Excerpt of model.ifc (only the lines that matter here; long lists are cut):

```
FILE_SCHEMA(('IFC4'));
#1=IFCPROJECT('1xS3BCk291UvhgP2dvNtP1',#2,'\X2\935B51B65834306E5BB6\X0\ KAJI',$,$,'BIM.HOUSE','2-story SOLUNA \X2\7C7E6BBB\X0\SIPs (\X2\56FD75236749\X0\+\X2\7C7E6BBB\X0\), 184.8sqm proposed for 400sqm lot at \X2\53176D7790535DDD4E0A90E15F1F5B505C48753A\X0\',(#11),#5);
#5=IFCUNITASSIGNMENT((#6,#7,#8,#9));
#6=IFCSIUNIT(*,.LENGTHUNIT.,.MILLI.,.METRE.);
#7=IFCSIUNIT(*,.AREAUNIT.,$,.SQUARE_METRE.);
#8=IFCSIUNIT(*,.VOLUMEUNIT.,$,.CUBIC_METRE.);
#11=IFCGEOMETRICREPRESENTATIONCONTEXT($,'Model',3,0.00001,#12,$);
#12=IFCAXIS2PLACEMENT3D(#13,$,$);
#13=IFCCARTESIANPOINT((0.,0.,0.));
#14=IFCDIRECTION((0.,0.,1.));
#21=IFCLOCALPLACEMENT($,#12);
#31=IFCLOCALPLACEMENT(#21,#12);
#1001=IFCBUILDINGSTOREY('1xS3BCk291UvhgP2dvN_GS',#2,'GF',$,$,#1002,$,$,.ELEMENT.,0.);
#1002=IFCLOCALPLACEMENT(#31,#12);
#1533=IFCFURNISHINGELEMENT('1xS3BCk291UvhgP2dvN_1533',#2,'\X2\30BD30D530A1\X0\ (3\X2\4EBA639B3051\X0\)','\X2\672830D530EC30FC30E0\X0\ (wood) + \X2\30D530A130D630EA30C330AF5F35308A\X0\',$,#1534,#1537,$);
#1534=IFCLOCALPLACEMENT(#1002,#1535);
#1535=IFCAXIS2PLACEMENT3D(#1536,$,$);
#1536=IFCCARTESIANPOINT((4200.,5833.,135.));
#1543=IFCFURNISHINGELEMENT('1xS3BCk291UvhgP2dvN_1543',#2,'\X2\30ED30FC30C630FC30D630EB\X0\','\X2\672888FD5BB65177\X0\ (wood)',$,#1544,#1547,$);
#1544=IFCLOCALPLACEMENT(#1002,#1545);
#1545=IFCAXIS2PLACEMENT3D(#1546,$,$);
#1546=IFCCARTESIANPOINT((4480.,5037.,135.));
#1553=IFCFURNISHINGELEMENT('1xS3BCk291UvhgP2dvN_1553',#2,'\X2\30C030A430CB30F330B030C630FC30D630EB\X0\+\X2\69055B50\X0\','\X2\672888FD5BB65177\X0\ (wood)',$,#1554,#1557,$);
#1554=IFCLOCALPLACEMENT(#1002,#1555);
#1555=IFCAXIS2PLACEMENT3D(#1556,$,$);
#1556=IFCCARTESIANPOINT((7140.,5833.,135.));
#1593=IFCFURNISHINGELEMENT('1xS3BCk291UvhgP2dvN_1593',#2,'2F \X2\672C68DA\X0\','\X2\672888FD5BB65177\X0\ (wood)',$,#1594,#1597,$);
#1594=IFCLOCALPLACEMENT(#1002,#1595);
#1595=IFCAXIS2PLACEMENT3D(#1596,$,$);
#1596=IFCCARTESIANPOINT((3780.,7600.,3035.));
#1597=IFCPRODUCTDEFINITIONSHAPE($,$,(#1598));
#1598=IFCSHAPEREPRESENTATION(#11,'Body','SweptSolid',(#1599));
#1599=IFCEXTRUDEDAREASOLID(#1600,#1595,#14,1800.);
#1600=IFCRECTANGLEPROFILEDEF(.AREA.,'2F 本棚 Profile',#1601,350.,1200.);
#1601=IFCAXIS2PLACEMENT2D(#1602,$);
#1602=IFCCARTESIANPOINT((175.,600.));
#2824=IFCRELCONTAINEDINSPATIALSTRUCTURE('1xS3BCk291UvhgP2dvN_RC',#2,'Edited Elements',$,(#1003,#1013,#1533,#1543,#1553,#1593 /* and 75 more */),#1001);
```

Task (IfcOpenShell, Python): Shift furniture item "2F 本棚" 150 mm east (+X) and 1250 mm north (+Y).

```python
import ifcopenshell
import ifcopenshell.api.geometry
import ifcopenshell.util.placement

model = ifcopenshell.open("model.ifc")

item = model.by_guid("1xS3BCk291UvhgP2dvN_1593")
matrix = ifcopenshell.util.placement.get_local_placement(item.ObjectPlacement)
matrix[0, 3] += 150.0
matrix[1, 3] += 1250.0
ifcopenshell.api.geometry.edit_object_placement(model, product=item, matrix=matrix, is_si=False)

print(ifcopenshell.util.placement.get_local_placement(item.ObjectPlacement).round(3) + 0.0)

model.write("model-out.ifc")
```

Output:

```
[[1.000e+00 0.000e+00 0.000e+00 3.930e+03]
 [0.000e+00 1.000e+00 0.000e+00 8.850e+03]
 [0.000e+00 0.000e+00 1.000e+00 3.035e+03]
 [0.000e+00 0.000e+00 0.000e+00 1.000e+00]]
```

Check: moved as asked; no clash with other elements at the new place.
